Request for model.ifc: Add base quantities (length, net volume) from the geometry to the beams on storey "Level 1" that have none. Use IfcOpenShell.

First a look at what the model holds.

```python
import ifcopenshell
import ifcopenshell.util.element
import ifcopenshell.util.unit

model = ifcopenshell.open("model.ifc")
print(model.schema)
for unit_type in ("LENGTHUNIT", "AREAUNIT", "VOLUMEUNIT"):
    print(unit_type, ifcopenshell.util.unit.calculate_unit_scale(model, unit_type))
storey = next(s for s in model.by_type("IfcBuildingStorey") if s.Name == "Level 1")
beams = [e for e in ifcopenshell.util.element.get_decomposition(storey) if e.is_a("IfcBeam")]
for e in sorted(beams, key=lambda e: e.id()):
    print(e.id(), e.is_a(), e.Name, list(ifcopenshell.util.element.get_psets(e, qtos_only=True)), sep=" | ")
```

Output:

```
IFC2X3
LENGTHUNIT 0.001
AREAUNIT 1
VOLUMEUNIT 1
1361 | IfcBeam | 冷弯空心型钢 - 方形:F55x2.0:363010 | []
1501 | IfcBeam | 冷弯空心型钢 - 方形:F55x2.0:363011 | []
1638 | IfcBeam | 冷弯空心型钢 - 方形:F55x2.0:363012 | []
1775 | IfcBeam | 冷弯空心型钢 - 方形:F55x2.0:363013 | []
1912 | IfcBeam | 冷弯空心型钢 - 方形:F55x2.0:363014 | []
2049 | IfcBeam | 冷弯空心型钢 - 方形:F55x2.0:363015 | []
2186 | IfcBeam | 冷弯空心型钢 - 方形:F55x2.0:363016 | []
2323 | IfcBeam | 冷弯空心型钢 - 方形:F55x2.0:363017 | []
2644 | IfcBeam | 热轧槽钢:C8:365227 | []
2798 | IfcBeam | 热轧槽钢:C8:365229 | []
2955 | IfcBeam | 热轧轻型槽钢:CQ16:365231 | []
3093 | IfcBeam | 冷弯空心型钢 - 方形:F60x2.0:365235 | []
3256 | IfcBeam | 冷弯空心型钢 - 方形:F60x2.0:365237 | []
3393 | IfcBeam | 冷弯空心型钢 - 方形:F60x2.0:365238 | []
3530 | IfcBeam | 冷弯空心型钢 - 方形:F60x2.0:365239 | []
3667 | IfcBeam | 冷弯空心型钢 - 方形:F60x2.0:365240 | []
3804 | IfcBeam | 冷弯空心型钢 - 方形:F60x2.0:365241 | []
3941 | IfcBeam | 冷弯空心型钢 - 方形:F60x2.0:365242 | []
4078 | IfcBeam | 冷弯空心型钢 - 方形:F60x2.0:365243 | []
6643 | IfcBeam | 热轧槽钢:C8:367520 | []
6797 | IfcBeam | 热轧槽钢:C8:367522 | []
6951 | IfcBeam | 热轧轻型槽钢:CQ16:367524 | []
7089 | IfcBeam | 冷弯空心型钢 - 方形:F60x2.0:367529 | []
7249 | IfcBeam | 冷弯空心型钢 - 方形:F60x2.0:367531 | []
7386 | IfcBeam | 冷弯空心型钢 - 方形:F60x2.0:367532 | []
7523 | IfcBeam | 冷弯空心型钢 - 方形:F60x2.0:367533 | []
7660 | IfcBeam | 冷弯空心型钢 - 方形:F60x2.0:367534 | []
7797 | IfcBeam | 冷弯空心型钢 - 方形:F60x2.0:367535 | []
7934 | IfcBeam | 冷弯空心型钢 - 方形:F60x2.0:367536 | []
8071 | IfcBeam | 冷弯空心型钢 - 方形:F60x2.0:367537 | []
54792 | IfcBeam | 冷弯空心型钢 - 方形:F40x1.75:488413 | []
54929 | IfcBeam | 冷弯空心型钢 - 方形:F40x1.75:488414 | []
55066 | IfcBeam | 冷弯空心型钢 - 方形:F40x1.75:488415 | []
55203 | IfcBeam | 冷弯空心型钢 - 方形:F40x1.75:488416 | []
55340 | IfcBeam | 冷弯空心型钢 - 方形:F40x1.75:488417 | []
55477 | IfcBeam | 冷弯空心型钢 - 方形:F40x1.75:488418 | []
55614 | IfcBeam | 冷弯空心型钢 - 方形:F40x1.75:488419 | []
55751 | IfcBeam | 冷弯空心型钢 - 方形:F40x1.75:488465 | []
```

```python
import ifcopenshell
import ifcopenshell.api.pset
import ifcopenshell.geom
import ifcopenshell.util.element
import ifcopenshell.util.shape
import ifcopenshell.util.unit

model = ifcopenshell.open("model.ifc")
unit_scale = ifcopenshell.util.unit.calculate_unit_scale(model)
volume_scale = ifcopenshell.util.unit.calculate_unit_scale(model, "VOLUMEUNIT")
settings = ifcopenshell.geom.settings()

storey = next(s for s in model.by_type("IfcBuildingStorey") if s.Name == "Level 1")
beams = [e for e in ifcopenshell.util.element.get_decomposition(storey) if e.is_a("IfcBeam")]

for e in sorted(beams, key=lambda e: e.id()):
    if ifcopenshell.util.element.get_psets(e, qtos_only=True, should_inherit=False):
        continue
    # Geometry comes back in metres, in the element's own axes.
    shape = ifcopenshell.geom.create_shape(settings, e)
    values = {
        "Length": ifcopenshell.util.shape.get_max_xyz(shape.geometry) / unit_scale,
        "NetVolume": ifcopenshell.util.shape.get_volume(shape.geometry) / volume_scale,
    }
    qto = ifcopenshell.api.pset.add_qto(model, product=e, name="BaseQuantities")
    ifcopenshell.api.pset.edit_qto(model, qto=qto, properties=values)
    print(e.id(), {k: round(v, 3) for k, v in values.items()})

model.write("model-out.ifc")
```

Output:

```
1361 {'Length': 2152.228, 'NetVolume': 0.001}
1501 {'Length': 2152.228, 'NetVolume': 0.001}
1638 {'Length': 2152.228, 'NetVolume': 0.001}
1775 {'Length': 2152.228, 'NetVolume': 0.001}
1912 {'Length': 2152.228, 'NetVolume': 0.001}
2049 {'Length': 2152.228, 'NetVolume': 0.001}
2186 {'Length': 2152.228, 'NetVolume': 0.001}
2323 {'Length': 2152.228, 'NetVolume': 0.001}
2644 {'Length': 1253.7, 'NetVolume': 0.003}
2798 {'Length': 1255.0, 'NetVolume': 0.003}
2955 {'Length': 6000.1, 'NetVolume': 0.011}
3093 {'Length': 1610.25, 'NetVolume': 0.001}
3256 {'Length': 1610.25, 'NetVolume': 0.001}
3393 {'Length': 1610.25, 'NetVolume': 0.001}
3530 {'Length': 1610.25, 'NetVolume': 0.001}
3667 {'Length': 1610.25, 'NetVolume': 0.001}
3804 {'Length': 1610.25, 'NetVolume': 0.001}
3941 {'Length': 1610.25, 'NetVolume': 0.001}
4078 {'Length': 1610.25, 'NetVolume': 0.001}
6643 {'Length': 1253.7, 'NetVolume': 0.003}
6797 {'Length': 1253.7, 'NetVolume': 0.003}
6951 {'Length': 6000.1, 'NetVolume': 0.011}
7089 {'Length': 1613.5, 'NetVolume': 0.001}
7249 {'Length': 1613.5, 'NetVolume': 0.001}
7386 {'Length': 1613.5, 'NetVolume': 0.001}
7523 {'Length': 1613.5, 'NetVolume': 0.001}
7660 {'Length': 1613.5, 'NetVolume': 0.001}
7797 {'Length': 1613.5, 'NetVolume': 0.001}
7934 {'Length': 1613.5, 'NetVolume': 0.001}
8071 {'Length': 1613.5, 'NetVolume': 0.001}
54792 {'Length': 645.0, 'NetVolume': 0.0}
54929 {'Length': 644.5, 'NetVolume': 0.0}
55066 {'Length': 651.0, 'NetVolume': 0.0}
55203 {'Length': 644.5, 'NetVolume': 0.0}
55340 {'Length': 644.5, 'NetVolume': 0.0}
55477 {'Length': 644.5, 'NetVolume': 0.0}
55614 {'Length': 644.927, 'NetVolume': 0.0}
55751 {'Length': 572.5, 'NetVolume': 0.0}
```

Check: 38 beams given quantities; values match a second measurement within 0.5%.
